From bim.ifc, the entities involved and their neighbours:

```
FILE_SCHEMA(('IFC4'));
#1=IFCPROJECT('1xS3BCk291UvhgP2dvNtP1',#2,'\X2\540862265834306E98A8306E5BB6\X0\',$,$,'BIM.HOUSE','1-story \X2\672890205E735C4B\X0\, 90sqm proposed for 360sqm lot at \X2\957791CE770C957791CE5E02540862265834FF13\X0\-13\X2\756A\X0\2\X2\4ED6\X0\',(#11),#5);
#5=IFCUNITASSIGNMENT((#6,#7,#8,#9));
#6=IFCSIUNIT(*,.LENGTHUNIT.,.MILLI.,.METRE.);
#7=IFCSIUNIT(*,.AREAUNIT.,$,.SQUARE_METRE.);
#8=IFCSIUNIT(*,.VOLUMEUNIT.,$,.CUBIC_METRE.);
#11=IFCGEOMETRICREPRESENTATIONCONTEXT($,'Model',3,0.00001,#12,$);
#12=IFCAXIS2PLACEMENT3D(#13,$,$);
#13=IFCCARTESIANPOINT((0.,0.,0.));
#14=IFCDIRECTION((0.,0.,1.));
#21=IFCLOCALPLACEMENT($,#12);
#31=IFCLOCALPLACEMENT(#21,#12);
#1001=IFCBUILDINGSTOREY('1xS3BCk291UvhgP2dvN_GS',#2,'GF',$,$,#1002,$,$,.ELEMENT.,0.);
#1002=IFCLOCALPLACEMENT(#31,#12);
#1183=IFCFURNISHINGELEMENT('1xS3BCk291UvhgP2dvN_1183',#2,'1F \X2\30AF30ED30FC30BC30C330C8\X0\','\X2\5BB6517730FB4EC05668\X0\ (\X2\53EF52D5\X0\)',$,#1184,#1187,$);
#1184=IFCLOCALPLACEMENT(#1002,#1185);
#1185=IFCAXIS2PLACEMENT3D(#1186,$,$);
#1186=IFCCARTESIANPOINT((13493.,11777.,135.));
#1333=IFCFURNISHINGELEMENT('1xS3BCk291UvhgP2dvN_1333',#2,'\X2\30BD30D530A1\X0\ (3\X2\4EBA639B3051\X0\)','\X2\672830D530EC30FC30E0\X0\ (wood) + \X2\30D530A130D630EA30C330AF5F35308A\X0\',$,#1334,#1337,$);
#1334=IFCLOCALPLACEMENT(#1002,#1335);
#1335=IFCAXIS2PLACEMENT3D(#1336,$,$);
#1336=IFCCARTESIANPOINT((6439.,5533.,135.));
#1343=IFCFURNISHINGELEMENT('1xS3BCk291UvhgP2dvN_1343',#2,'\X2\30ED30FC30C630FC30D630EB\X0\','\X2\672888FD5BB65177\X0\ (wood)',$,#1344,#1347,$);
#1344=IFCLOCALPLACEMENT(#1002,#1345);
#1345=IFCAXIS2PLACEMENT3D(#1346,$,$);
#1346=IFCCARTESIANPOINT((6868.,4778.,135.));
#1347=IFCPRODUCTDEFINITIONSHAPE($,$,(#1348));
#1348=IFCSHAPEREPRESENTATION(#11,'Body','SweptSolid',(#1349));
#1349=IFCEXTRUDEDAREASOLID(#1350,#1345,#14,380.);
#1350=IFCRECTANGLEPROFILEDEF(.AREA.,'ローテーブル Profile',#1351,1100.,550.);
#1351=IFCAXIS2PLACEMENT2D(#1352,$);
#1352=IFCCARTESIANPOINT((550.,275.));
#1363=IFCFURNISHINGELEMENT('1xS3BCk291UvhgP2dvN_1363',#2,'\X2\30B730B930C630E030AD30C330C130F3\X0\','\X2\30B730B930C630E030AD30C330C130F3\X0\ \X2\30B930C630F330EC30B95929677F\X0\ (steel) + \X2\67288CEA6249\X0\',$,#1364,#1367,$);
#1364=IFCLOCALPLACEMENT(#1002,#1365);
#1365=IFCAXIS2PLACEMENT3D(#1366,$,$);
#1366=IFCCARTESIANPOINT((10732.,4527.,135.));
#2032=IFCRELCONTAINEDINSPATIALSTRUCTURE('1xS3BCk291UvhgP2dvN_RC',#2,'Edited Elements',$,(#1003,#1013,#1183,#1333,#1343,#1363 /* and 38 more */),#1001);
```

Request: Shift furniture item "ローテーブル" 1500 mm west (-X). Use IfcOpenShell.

```python
import ifcopenshell
import ifcopenshell.api.geometry
import ifcopenshell.util.placement
import ifcopenshell.util.unit

model = ifcopenshell.open("bim.ifc")
unit_scale = ifcopenshell.util.unit.calculate_unit_scale(model)

item = model.by_guid("1xS3BCk291UvhgP2dvN_1343")
matrix = ifcopenshell.util.placement.get_local_placement(item.ObjectPlacement)
matrix[0, 3] -= 1.5 / unit_scale
ifcopenshell.api.geometry.edit_object_placement(model, product=item, matrix=matrix, is_si=False)

print(ifcopenshell.util.placement.get_local_placement(item.ObjectPlacement).round(3) + 0.0)

model.write("bim_rev.ifc")
```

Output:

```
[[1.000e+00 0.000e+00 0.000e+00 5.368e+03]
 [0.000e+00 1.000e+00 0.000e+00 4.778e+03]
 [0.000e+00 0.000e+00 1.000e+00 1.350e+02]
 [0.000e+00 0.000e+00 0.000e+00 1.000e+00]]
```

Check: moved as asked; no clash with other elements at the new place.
